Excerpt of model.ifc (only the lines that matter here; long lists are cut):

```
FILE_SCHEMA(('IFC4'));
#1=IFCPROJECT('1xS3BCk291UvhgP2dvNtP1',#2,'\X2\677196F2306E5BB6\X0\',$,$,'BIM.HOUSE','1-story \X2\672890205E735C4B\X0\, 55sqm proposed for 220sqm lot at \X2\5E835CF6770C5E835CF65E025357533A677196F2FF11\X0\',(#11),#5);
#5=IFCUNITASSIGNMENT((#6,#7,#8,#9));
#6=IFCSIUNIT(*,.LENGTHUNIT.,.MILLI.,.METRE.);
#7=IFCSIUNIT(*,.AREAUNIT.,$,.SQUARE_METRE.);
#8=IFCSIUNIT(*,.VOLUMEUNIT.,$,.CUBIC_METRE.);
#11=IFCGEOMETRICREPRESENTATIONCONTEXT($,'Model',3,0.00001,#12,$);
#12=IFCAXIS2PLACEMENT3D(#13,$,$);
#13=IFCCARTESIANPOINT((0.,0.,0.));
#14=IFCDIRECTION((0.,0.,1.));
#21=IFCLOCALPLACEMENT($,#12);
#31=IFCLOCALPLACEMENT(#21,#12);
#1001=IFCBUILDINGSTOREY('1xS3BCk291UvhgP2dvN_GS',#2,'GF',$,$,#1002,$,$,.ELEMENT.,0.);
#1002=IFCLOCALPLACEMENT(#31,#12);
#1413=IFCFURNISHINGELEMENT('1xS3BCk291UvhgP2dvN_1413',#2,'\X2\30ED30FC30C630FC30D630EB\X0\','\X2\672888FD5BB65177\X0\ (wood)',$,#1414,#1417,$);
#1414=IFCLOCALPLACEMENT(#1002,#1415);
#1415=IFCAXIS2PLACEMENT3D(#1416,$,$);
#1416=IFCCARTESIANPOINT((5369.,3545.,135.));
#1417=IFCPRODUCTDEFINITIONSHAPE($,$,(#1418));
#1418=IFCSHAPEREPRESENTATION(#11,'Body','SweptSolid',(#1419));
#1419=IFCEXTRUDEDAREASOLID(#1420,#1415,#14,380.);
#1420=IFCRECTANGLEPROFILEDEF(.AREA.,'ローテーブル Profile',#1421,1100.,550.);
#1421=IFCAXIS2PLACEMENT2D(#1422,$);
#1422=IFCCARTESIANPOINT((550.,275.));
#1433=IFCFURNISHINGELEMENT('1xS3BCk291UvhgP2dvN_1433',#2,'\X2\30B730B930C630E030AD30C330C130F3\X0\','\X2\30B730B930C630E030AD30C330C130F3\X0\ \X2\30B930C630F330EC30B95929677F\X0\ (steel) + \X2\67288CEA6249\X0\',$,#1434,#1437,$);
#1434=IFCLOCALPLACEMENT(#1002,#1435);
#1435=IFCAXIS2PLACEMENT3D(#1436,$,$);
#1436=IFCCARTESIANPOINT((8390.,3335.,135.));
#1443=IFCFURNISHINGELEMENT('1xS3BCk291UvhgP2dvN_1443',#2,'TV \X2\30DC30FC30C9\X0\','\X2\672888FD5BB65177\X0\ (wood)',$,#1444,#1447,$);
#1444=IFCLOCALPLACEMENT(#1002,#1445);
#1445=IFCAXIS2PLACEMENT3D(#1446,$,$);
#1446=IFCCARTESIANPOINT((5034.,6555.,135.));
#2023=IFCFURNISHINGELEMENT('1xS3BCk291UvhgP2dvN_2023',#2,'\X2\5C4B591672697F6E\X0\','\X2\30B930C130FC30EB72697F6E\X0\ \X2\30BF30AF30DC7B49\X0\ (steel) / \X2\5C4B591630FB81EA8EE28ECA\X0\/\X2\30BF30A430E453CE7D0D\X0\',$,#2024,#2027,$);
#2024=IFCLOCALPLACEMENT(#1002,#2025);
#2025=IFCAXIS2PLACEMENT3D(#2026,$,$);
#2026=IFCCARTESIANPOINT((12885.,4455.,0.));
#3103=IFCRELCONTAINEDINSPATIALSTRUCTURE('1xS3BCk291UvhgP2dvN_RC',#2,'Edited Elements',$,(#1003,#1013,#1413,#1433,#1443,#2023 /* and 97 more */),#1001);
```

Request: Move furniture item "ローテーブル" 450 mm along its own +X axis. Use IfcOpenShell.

```python
import ifcopenshell
import ifcopenshell.api.geometry
import ifcopenshell.util.placement
import ifcopenshell.util.unit

model = ifcopenshell.open("model.ifc")
unit_scale = ifcopenshell.util.unit.calculate_unit_scale(model)

item = model.by_guid("1xS3BCk291UvhgP2dvN_1413")
matrix = ifcopenshell.util.placement.get_local_placement(item.ObjectPlacement)
matrix[:3, 3] += matrix[:3, 0] * 0.45 / unit_scale
ifcopenshell.api.geometry.edit_object_placement(model, product=item, matrix=matrix, is_si=False)

print(ifcopenshell.util.placement.get_local_placement(item.ObjectPlacement).round(3) + 0.0)

model.write("model_edited.ifc")
```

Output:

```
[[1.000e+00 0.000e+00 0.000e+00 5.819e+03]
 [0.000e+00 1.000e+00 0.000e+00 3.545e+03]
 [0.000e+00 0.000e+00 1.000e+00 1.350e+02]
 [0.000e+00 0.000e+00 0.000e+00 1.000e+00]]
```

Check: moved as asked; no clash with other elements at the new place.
